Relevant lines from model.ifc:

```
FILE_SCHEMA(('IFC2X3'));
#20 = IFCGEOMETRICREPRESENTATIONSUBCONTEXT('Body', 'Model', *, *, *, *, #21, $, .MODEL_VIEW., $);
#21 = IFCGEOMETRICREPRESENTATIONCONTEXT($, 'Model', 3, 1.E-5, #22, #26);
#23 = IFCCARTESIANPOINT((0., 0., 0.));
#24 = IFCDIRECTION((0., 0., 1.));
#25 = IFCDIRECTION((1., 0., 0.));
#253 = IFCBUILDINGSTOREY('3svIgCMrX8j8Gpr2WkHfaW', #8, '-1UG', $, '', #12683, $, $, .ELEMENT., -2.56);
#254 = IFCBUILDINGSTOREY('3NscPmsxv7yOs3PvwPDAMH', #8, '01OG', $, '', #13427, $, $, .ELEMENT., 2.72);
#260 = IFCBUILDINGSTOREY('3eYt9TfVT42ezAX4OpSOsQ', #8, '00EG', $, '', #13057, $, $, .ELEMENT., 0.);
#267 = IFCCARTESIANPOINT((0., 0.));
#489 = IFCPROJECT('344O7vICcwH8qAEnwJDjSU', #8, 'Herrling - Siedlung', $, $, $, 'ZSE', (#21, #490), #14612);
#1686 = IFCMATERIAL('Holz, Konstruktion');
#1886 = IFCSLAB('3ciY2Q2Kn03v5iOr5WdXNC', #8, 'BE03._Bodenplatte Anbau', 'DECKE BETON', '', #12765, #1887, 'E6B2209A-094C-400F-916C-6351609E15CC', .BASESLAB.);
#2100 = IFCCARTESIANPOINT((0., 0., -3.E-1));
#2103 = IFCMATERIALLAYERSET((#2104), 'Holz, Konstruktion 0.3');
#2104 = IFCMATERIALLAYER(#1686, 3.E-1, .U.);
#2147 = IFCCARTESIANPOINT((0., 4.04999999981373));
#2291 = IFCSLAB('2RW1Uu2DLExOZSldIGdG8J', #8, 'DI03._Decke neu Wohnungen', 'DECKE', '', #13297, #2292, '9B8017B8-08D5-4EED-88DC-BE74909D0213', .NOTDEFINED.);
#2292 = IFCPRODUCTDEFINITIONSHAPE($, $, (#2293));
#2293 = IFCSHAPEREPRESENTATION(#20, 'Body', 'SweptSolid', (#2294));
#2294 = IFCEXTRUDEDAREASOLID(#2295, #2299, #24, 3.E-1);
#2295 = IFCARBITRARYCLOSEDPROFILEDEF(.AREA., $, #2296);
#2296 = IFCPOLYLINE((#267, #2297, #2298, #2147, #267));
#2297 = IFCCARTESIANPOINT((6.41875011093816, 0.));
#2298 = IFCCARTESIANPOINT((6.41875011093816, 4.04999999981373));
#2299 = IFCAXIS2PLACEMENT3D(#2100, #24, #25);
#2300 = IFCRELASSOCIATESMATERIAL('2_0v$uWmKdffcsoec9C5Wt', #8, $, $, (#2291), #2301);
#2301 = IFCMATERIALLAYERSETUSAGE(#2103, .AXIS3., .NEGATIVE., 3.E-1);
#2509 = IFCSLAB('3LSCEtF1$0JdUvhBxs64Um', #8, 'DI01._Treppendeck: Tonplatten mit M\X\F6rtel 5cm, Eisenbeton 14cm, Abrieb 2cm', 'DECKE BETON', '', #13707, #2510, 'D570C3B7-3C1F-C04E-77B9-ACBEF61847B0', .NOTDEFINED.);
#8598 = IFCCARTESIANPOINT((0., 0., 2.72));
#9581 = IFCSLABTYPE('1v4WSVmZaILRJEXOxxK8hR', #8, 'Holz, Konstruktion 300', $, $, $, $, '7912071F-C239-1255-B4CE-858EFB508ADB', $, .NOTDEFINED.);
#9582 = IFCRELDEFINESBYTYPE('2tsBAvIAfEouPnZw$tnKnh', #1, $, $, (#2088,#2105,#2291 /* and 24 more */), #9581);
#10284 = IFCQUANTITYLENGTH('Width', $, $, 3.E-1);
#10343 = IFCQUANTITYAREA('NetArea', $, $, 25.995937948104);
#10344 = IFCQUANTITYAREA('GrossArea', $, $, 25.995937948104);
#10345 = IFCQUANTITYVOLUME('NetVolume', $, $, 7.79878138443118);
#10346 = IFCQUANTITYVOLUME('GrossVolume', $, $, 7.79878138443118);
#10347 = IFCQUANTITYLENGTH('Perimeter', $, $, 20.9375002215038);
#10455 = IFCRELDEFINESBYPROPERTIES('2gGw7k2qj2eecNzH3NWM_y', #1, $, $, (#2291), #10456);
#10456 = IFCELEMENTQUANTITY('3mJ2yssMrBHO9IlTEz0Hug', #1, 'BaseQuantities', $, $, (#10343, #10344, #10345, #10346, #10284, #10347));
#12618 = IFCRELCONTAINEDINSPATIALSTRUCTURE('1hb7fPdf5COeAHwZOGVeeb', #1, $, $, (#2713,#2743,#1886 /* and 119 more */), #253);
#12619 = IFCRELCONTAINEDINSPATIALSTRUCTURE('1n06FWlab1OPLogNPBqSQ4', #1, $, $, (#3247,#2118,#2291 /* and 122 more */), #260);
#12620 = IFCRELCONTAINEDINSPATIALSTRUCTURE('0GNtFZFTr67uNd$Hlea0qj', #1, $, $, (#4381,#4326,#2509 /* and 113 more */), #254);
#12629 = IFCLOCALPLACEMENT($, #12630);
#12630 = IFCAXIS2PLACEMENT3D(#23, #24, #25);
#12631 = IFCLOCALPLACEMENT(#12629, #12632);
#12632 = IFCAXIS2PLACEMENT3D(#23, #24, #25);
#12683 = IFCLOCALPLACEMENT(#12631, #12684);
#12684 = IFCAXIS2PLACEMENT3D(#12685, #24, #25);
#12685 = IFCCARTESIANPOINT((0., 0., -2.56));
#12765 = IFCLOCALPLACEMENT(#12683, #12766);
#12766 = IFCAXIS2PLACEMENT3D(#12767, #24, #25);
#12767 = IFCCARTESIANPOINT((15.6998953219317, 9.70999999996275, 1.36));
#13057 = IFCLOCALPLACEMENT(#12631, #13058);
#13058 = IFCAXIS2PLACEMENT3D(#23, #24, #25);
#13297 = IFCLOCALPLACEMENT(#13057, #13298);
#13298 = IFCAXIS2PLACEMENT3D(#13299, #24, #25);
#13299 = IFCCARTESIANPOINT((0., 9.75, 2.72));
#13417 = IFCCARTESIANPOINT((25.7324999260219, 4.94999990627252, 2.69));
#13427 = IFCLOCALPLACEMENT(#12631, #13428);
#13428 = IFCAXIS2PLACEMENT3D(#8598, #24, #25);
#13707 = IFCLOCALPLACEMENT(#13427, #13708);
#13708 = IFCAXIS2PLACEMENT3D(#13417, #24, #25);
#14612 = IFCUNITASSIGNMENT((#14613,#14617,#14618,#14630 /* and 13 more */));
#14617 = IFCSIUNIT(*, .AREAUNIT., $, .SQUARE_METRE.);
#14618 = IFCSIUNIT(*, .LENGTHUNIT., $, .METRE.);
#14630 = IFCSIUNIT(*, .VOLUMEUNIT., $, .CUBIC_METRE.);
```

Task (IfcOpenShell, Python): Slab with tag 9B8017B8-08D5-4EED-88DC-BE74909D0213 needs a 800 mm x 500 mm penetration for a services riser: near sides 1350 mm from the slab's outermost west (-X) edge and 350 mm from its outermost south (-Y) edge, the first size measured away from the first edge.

```python
import numpy as np
import ifcopenshell
import ifcopenshell.api.feature
import ifcopenshell.api.geometry
import ifcopenshell.api.pset
import ifcopenshell.api.root
import ifcopenshell.geom
import ifcopenshell.util.element
import ifcopenshell.util.placement
import ifcopenshell.util.representation
import ifcopenshell.util.shape
import ifcopenshell.util.unit

model = ifcopenshell.open("model.ifc")
unit_scale = ifcopenshell.util.unit.calculate_unit_scale(model)
area_scale = ifcopenshell.util.unit.calculate_unit_scale(model, "AREAUNIT")
volume_scale = ifcopenshell.util.unit.calculate_unit_scale(model, "VOLUMEUNIT")
settings = ifcopenshell.geom.settings()


def volume(element):
    """Net volume in cubic metres, openings subtracted."""
    shape = ifcopenshell.geom.create_shape(settings, element)
    return ifcopenshell.util.shape.get_volume(shape.geometry)


slab = model.by_id(2291)
before = volume(slab)

# Extent in the slab's own axes, in metres. The edges named are its -X and -Y sides.
slab_shape = ifcopenshell.geom.create_shape(settings, slab)
vertices = ifcopenshell.util.shape.get_vertices(slab_shape.geometry)
x_min, y_min, bottom = vertices.min(axis=0)
top = vertices[:, 2].max()

opening = ifcopenshell.api.root.create_entity(model, ifc_class="IfcOpeningElement", name="Services riser opening")
context = ifcopenshell.util.representation.get_context(model, "Model", "Body", "MODEL_VIEW")
width, depth = 0.8, 0.5
outline = [(0.0, 0.0), (width, 0.0), (width, depth), (0.0, depth), (0.0, 0.0)]
# Overshoot both faces by 50 mm so the cut is clean.
shape = ifcopenshell.api.geometry.add_slab_representation(
    model, context=context, depth=top - bottom + 0.1, polyline=outline
)
ifcopenshell.api.geometry.assign_representation(model, product=opening, representation=shape)

matrix = ifcopenshell.util.placement.get_local_placement(slab.ObjectPlacement)
matrix[:, 3] = matrix @ np.append(np.array([x_min + 1.35, y_min + 0.35, bottom - 0.05]) / unit_scale, 1.0)
ifcopenshell.api.geometry.edit_object_placement(model, product=opening, matrix=matrix, is_si=False)
ifcopenshell.api.feature.add_feature(model, feature=opening, element=slab)

after = volume(slab)

# Update the slab's stored quantities.
qto = model.by_id(ifcopenshell.util.element.get_pset(slab, "BaseQuantities", should_inherit=False)["id"])
ifcopenshell.api.pset.edit_qto(model, qto=qto, properties={
    "NetArea": after / (top - bottom) / area_scale,
    "NetVolume": after / volume_scale,
})

print(f"slab volume {before:.3f} -> {after:.3f} m3")

model.write("model_v2.ifc")
```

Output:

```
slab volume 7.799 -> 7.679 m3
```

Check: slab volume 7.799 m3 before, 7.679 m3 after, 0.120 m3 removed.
